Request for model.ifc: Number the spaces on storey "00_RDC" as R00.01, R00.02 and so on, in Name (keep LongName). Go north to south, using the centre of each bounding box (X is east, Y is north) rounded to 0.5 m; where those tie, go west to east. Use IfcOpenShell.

First a look at what the model holds.

```python
import ifcopenshell
import ifcopenshell.util.element
import ifcopenshell.util.placement

model = ifcopenshell.open("model.ifc")
print(model.schema)
storey = next(s for s in model.by_type("IfcBuildingStorey") if s.Name == "00_RDC")
spaces = [e for e in ifcopenshell.util.element.get_decomposition(storey) if e.is_a("IfcSpace")]
for e in sorted(spaces, key=lambda e: e.id()):
    origin = ifcopenshell.util.placement.get_local_placement(e.ObjectPlacement)[:3, 3]
    print(e.id(), e.Name, e.LongName, origin.round(2) + 0.0, sep=" | ")
```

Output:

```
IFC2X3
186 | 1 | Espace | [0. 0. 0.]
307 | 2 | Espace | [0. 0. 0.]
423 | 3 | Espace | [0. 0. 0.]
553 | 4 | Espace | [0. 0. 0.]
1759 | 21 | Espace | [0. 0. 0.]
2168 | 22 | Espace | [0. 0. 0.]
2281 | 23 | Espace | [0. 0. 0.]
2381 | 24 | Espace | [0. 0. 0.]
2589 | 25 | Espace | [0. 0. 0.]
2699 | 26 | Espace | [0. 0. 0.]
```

```python
import ifcopenshell
import ifcopenshell.geom
import ifcopenshell.util.element
import ifcopenshell.util.shape

model = ifcopenshell.open("model.ifc")
settings = ifcopenshell.geom.settings()
settings.set("use-world-coords", True)


def centre(element):
    shape = ifcopenshell.geom.create_shape(settings, element)
    return ifcopenshell.util.shape.get_bbox_centroid(shape.geometry)


storey = next(s for s in model.by_type("IfcBuildingStorey") if s.Name == "00_RDC")
spaces = [e for e in ifcopenshell.util.element.get_decomposition(storey) if e.is_a("IfcSpace")]

# Insertion points can sit at a corner or the storey origin, so sort by the geometry (in metres).
centres = {e: centre(e) for e in spaces}
spaces.sort(key=lambda e: (-round(centres[e][1] / 0.5), centres[e][0]))

for i, e in enumerate(spaces, start=1):
    number = f"R00.{i:02d}"
    e.Name = number
    print(e.id(), number)

model.write("model_v2.ifc")
```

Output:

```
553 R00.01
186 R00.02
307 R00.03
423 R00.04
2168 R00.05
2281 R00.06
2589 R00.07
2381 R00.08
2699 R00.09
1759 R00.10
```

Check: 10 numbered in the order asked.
